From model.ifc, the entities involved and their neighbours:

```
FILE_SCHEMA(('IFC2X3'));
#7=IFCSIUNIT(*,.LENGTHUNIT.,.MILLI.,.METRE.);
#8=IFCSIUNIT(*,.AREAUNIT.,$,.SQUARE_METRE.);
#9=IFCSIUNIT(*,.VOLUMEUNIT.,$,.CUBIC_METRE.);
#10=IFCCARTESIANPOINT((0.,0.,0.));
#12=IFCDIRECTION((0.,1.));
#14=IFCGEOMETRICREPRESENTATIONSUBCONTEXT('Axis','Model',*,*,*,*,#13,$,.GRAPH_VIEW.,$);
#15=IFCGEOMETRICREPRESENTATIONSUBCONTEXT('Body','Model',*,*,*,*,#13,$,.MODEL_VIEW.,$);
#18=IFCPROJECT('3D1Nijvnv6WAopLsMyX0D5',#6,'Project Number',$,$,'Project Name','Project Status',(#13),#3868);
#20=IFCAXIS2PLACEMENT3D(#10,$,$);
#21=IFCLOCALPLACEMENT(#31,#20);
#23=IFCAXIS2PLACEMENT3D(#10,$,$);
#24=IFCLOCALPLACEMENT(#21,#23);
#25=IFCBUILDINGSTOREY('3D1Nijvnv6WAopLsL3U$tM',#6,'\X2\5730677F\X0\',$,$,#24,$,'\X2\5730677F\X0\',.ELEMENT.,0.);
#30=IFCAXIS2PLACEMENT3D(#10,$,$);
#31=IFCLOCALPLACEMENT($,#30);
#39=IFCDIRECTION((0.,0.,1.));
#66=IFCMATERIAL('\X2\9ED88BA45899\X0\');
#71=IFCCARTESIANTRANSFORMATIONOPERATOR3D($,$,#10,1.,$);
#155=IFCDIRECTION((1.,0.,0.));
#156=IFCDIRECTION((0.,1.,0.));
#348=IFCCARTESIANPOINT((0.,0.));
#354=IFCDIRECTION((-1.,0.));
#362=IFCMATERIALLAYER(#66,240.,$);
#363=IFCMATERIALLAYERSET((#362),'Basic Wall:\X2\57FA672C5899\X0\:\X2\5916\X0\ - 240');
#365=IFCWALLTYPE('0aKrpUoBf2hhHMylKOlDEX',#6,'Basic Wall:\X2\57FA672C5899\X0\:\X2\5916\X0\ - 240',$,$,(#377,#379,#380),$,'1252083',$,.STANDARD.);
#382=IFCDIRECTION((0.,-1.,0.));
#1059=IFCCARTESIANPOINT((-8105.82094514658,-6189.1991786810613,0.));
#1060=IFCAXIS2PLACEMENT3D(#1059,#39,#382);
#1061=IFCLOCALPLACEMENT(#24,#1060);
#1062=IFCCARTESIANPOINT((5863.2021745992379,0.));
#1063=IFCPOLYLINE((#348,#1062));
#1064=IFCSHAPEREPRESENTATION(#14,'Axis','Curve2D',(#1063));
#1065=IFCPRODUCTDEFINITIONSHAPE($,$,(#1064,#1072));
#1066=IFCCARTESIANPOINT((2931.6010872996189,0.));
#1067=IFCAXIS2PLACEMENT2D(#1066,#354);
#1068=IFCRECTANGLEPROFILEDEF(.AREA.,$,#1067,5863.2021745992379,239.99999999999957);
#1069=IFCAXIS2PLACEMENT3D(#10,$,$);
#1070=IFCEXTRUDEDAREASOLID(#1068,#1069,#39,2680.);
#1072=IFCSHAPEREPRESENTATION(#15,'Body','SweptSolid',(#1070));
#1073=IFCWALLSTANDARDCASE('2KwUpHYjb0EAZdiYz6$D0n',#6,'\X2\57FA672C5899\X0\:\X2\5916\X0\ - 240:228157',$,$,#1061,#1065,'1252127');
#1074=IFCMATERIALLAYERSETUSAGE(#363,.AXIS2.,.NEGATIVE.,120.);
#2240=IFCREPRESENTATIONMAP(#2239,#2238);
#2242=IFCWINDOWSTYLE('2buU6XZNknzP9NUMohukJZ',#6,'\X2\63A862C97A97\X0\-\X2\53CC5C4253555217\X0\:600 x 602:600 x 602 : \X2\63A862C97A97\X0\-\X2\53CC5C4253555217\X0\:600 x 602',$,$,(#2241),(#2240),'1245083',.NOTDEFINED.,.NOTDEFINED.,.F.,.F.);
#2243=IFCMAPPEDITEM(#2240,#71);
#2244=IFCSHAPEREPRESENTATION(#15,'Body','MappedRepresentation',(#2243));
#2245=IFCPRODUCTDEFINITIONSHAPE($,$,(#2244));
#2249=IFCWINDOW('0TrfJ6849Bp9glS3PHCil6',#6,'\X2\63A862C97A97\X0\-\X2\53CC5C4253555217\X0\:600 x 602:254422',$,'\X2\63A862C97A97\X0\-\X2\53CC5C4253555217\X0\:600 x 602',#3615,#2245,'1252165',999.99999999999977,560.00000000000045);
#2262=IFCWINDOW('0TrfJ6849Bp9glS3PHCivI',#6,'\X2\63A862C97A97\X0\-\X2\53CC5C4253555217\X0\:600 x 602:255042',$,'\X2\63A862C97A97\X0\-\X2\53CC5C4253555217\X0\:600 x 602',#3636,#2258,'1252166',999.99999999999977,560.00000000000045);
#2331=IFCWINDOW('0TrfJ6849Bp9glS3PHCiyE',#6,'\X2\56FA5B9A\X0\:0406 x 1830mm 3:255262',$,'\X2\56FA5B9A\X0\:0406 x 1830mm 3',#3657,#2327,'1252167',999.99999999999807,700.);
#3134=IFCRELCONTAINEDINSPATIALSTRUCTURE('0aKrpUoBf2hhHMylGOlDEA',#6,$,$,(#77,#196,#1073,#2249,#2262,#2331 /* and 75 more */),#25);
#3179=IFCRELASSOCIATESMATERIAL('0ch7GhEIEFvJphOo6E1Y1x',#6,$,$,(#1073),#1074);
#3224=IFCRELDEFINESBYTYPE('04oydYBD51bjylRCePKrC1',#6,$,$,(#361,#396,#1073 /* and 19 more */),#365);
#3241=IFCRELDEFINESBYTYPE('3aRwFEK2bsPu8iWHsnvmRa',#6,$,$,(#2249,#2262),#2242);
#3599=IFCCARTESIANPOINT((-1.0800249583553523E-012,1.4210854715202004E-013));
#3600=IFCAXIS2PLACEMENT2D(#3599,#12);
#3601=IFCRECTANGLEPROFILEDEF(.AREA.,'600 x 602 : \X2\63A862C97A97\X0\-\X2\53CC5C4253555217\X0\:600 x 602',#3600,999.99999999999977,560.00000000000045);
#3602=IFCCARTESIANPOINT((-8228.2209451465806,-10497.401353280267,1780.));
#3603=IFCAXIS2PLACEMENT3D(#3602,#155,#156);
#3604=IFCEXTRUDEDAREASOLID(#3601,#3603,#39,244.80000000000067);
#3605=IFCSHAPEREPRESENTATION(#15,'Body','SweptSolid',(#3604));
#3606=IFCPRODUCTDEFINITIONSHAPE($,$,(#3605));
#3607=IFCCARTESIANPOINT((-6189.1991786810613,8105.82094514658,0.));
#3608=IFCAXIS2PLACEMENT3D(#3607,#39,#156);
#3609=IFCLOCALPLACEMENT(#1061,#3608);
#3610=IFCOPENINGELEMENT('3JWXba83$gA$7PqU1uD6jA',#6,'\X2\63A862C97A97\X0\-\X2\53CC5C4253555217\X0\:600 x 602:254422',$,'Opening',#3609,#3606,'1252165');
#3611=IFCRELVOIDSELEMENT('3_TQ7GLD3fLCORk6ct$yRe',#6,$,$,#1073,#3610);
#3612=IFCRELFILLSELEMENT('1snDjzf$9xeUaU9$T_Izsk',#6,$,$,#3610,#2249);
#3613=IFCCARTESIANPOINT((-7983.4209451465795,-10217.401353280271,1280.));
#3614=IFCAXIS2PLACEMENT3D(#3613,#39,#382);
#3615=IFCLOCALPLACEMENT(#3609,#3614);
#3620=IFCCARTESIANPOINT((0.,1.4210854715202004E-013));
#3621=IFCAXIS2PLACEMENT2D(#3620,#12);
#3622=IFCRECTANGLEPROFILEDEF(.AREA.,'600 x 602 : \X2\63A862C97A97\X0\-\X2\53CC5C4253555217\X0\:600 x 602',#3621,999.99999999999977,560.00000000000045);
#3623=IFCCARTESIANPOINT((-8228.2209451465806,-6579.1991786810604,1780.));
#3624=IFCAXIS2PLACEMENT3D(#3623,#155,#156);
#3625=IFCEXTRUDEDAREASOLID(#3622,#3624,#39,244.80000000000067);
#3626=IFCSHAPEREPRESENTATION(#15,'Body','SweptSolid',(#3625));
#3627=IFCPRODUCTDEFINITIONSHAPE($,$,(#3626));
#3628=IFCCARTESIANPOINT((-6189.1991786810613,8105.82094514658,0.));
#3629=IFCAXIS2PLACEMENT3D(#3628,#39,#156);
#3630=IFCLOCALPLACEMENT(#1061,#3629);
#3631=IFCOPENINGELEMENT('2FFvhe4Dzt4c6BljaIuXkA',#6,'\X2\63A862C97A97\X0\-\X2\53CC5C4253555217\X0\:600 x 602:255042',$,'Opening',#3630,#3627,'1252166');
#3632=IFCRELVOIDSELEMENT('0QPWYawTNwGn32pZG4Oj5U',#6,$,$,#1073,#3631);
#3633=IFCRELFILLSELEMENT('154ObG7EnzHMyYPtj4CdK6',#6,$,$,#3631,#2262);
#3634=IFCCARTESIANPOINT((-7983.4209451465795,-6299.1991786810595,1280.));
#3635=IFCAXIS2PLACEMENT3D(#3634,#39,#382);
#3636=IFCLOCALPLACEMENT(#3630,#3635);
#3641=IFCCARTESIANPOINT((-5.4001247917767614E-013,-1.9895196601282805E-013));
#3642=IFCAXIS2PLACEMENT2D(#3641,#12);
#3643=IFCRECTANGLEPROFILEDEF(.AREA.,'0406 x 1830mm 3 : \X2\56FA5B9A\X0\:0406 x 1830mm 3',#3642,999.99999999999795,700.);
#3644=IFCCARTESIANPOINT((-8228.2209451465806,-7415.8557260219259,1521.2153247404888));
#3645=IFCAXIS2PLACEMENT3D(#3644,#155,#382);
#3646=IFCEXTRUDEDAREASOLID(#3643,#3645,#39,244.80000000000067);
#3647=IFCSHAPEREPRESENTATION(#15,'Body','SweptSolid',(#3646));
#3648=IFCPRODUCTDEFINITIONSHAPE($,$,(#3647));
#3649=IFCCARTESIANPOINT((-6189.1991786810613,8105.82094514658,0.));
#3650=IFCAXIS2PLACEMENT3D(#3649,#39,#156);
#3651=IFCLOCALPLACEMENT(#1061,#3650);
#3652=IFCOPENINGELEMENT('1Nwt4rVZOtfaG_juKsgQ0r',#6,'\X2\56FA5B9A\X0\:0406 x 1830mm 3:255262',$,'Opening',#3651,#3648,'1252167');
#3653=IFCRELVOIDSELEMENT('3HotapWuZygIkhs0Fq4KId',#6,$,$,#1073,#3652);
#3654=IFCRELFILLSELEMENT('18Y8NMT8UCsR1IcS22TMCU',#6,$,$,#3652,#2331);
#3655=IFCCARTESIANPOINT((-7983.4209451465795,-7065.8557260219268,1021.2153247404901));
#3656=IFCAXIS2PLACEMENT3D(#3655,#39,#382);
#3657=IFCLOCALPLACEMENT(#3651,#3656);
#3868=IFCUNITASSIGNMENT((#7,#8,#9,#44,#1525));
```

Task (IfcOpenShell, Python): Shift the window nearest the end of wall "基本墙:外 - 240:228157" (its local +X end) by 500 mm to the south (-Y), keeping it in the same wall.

```python
import ifcopenshell
import ifcopenshell.api.geometry
import ifcopenshell.util.placement

model = ifcopenshell.open("model.ifc")

window = model.by_id(2249)
opening = window.FillsVoids[0].RelatingOpeningElement
wall = opening.VoidsElements[0].RelatingBuildingElement

wall_matrix = ifcopenshell.util.placement.get_local_placement(wall.ObjectPlacement)
shift = wall_matrix[:3, 0] * 500.0
before = ifcopenshell.util.placement.get_local_placement(window.ObjectPlacement)[:3, 3].copy()

# The window is placed relative to its opening, so it follows when the opening moves.
matrix = ifcopenshell.util.placement.get_local_placement(opening.ObjectPlacement)
matrix[:3, 3] += shift
ifcopenshell.api.geometry.edit_object_placement(
    model, product=opening, matrix=matrix, is_si=False, should_transform_children=True
)

after = ifcopenshell.util.placement.get_local_placement(window.ObjectPlacement)[:3, 3]
print("window moved by", (after - before).round(3) + 0.0)

model.write("model_v2.ifc")
```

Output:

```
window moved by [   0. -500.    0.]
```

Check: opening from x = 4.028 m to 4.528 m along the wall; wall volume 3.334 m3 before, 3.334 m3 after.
